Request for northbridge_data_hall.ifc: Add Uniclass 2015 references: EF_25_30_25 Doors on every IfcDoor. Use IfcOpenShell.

First a look at what the model holds.

```python
import ifcopenshell

model = ifcopenshell.open("northbridge_data_hall.ifc")
print(model.schema)
print("classifications:", [c.Name for c in model.by_type("IfcClassification")])
for ifc_class in ("IfcDoor", "IfcRoof", "IfcStair", "IfcWall", "IfcWindow"):
    print(ifc_class, len(model.by_type(ifc_class)))
```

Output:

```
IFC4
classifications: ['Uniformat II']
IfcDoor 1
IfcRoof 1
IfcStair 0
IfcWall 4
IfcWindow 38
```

```python
import ifcopenshell
import ifcopenshell.api.classification

model = ifcopenshell.open("northbridge_data_hall.ifc")

system = ifcopenshell.api.classification.add_classification(model, classification="Uniclass 2015")

codes = {
    "IfcDoor": ("EF_25_30_25", "Doors"),
}
for ifc_class, (code, name) in codes.items():
    products = model.by_type(ifc_class)
    ifcopenshell.api.classification.add_reference(
        model, products=products, classification=system, identification=code, name=name
    )
    print(code, len(products))

model.write("northbridge_data_hall-out.ifc")
```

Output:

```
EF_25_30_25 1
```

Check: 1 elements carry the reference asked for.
